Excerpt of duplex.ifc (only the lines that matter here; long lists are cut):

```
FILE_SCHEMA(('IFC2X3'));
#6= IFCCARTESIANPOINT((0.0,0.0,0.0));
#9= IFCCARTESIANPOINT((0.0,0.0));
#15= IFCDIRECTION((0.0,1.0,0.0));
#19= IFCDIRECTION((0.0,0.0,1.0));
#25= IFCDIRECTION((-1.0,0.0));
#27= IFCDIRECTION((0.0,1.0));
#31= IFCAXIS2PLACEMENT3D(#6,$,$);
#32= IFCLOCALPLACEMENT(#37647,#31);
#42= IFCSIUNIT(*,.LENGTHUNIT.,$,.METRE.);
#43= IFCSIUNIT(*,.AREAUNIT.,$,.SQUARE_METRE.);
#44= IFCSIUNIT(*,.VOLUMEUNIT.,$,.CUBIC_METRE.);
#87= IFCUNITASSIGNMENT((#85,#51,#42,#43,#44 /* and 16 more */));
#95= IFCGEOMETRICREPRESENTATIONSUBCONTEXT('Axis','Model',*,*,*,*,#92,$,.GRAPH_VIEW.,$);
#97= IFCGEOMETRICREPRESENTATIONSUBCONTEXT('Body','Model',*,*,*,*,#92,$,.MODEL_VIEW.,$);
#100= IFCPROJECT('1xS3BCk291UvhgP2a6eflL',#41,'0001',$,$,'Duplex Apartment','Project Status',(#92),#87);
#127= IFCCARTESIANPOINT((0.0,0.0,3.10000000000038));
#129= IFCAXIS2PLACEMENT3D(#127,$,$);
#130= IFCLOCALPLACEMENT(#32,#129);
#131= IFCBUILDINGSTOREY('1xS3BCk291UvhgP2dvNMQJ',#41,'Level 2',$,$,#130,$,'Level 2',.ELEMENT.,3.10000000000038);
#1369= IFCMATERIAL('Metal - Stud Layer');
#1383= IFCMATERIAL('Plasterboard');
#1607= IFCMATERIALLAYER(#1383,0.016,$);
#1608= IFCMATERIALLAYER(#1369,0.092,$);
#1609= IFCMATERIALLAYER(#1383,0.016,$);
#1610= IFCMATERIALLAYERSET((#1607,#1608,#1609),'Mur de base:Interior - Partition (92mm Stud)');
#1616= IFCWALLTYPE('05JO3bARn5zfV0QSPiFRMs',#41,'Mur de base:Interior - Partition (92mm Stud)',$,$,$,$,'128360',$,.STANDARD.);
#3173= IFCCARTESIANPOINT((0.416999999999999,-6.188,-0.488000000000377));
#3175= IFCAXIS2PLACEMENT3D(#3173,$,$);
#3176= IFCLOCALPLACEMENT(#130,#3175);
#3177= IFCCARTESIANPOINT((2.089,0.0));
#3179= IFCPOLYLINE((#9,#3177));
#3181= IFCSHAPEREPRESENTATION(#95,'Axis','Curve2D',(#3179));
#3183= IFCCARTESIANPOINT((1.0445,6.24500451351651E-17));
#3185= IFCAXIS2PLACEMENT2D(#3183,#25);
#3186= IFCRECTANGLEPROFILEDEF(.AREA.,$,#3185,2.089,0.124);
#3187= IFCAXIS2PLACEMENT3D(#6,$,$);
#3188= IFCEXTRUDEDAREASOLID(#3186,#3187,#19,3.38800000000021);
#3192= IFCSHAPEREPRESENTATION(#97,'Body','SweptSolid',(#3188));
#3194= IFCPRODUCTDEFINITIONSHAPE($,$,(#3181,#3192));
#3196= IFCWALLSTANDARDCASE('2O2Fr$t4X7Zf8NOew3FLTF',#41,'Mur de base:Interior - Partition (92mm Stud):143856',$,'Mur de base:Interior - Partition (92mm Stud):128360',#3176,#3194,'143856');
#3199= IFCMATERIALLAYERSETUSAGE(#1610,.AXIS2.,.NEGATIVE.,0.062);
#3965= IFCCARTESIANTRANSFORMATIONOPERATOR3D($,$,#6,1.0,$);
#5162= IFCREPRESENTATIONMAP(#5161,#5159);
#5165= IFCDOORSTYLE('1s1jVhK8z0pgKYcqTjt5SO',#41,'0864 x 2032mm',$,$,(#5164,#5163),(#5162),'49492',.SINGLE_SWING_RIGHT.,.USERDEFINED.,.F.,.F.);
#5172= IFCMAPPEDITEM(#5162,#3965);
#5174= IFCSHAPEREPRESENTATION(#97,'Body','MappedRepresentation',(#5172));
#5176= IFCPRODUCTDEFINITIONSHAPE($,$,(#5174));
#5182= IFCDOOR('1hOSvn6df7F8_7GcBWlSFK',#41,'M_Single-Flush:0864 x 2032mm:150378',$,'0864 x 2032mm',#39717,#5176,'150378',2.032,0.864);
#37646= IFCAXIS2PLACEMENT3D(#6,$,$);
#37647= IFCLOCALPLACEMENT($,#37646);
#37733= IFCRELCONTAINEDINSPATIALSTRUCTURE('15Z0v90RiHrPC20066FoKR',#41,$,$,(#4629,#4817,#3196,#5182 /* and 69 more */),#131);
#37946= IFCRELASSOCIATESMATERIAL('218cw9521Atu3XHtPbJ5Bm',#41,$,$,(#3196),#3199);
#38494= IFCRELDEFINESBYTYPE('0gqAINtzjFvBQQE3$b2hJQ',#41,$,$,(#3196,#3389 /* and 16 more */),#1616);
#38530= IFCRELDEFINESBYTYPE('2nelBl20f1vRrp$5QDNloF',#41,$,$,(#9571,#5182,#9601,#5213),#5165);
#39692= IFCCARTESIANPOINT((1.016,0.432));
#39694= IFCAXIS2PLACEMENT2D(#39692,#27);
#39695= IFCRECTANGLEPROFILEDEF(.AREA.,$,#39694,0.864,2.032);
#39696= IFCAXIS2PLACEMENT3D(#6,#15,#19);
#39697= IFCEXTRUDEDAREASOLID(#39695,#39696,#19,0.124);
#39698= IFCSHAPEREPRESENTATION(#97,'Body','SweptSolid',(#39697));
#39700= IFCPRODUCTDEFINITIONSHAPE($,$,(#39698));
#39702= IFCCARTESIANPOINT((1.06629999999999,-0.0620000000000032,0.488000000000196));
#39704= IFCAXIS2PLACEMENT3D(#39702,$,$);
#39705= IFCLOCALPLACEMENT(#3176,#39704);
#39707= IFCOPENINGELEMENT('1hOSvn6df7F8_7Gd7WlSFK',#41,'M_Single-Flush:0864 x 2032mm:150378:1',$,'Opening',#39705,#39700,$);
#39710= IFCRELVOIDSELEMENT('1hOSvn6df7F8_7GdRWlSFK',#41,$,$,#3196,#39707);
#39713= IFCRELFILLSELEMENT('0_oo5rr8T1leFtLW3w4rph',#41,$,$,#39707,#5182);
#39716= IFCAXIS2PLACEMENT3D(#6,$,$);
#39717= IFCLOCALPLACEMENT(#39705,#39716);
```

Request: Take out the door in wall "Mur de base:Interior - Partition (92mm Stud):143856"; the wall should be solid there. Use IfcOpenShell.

```python
import ifcopenshell
import ifcopenshell.api.feature
import ifcopenshell.api.root
import ifcopenshell.geom
import ifcopenshell.util.shape

model = ifcopenshell.open("duplex.ifc")
settings = ifcopenshell.geom.settings()


def volume(element):
    """Net volume in cubic metres, openings subtracted."""
    shape = ifcopenshell.geom.create_shape(settings, element)
    return ifcopenshell.util.shape.get_volume(shape.geometry)


door = model.by_guid("1hOSvn6df7F8_7GcBWlSFK")
opening = door.FillsVoids[0].RelatingOpeningElement
wall = opening.VoidsElements[0].RelatingBuildingElement
before = volume(wall)

ifcopenshell.api.root.remove_product(model, product=door)
ifcopenshell.api.feature.remove_feature(model, feature=opening)

after = volume(wall)

print(f"wall volume {before:.3f} -> {after:.3f} m3")

model.write("duplex_edited.ifc")
```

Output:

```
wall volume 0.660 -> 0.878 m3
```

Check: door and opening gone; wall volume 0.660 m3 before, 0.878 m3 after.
